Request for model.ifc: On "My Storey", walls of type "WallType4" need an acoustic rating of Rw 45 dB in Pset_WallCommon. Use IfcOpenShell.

First a look at what the model holds.

```python
import ifcopenshell
import ifcopenshell.util.element

model = ifcopenshell.open("model.ifc")
print(model.schema)
storey = next(s for s in model.by_type("IfcBuildingStorey") if s.Name == "My Storey")
walls = [e for e in ifcopenshell.util.element.get_decomposition(storey) if e.is_a("IfcWall")]
seen = {}
for e in walls:
    element_type = ifcopenshell.util.element.get_type(e)
    key = (element_type.Name if element_type != e and element_type else None, ifcopenshell.util.element.get_pset(e, "Pset_WallCommon", "AcousticRating"))
    seen[key] = seen.get(key, 0) + 1
for (name, value), count in sorted(seen.items(), key=str):
    print(count, "x", name, "|", value)
```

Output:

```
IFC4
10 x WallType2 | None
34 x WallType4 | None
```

```python
import ifcopenshell
import ifcopenshell.api.pset
import ifcopenshell.util.element

model = ifcopenshell.open("model.ifc")

storey = next(s for s in model.by_type("IfcBuildingStorey") if s.Name == "My Storey")
walls = [e for e in ifcopenshell.util.element.get_decomposition(storey) if e.is_a("IfcWall")]

count = 0
for e in walls:
    element_type = ifcopenshell.util.element.get_type(e)
    if element_type in (None, e) or element_type.Name != "WallType4":
        continue
    # add_pset returns the element's existing set when there is one.
    pset = ifcopenshell.api.pset.add_pset(model, product=e, name="Pset_WallCommon")
    ifcopenshell.api.pset.edit_pset(model, pset=pset, properties={"AcousticRating": "Rw 45 dB"})
    count += 1

print(count, "walls updated")

model.write("model_rev.ifc")
```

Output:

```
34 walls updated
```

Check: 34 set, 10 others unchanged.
